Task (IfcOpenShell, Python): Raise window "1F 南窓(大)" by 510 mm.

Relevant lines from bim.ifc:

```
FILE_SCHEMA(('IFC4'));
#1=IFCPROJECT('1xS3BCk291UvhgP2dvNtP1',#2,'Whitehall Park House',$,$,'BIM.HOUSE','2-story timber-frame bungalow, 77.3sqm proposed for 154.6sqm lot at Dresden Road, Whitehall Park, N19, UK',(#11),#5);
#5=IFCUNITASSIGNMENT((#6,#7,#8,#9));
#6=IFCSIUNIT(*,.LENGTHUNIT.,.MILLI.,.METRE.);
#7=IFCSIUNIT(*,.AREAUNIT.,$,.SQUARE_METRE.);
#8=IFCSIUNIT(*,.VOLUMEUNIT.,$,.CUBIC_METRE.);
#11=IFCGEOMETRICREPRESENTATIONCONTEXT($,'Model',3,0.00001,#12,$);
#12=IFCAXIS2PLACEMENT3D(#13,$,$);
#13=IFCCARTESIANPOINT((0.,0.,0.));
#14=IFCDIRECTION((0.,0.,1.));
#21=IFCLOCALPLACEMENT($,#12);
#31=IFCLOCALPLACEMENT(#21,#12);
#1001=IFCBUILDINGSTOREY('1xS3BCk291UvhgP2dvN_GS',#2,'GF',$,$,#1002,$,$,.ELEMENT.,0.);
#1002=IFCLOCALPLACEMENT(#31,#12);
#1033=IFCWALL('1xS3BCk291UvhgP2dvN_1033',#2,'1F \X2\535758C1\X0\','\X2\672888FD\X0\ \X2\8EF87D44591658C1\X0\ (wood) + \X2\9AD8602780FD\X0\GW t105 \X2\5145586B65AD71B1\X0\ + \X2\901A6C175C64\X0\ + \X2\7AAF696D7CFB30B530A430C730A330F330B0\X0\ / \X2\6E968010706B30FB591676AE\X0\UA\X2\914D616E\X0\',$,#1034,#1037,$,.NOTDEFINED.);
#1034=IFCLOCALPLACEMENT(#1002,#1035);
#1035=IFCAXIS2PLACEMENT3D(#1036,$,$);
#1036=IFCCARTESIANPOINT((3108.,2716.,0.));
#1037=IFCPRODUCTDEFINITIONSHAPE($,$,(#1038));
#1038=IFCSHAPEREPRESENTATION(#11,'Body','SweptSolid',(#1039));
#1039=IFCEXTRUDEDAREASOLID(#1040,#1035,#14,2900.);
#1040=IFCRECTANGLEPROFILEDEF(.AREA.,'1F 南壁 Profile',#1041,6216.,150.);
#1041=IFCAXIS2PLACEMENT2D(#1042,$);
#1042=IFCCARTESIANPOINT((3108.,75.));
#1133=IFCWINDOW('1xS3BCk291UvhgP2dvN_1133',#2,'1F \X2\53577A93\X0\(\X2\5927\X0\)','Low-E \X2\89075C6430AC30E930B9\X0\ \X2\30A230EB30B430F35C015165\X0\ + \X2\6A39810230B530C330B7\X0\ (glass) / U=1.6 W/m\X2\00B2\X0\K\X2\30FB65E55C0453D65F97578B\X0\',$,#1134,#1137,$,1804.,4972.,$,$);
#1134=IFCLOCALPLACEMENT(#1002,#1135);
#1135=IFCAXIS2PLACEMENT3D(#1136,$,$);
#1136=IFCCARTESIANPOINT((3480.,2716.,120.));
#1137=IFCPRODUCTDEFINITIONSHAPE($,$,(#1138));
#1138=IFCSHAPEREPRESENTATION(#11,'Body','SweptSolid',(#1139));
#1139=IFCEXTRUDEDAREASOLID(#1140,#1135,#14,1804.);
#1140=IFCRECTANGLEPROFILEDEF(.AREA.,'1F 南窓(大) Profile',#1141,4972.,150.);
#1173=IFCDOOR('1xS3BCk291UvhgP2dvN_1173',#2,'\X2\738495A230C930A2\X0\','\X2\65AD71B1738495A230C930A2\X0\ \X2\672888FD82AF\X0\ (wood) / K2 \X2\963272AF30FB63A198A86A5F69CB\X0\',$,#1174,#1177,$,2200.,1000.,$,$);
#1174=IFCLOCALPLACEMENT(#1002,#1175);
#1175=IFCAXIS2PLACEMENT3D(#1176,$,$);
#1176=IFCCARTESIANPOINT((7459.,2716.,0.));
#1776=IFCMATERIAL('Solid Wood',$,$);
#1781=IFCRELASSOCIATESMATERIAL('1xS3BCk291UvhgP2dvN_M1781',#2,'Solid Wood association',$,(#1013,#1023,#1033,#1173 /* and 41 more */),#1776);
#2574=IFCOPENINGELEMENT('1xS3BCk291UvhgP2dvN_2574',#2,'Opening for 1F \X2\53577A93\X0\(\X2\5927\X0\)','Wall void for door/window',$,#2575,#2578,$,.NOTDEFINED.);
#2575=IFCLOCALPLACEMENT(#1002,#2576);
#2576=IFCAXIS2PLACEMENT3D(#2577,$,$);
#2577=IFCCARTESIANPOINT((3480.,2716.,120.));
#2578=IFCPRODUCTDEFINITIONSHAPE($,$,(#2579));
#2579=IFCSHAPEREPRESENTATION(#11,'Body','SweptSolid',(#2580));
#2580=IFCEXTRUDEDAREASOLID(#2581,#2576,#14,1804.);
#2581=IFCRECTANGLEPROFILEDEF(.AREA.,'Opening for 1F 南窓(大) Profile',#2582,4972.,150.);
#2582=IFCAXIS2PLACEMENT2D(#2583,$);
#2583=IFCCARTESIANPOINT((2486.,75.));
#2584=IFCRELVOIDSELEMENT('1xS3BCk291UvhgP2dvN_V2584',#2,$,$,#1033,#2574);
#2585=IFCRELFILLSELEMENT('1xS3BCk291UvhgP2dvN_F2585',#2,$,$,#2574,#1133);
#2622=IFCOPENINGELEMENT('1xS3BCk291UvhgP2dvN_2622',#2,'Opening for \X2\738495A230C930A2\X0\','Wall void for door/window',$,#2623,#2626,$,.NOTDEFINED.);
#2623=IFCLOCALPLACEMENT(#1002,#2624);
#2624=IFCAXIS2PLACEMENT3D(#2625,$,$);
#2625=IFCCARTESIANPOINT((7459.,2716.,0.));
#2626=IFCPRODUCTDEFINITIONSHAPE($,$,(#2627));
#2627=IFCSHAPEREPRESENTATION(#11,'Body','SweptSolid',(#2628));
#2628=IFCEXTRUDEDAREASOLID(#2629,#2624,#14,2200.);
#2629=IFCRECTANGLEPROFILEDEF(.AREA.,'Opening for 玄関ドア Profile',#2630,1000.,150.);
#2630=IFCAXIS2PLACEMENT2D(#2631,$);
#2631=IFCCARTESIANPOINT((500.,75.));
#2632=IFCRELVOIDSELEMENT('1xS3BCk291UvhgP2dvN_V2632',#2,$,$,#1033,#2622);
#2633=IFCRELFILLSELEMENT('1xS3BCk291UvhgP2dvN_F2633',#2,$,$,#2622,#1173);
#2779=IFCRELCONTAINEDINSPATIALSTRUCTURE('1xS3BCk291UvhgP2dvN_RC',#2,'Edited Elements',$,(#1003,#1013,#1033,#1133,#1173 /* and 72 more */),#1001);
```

```python
import numpy as np
import ifcopenshell
import ifcopenshell.api.geometry
import ifcopenshell.util.placement
import ifcopenshell.util.unit

model = ifcopenshell.open("bim.ifc")
unit_scale = ifcopenshell.util.unit.calculate_unit_scale(model)

window = model.by_guid("1xS3BCk291UvhgP2dvN_1133")
opening = window.FillsVoids[0].RelatingOpeningElement
dz = 0.51 / unit_scale

shift = np.array([0.0, 0.0, dz])
# The window is not placed relative to its opening, so move both.
for product in (opening, window):
    matrix = ifcopenshell.util.placement.get_local_placement(product.ObjectPlacement)
    matrix[:3, 3] += shift
    ifcopenshell.api.geometry.edit_object_placement(model, product=product, matrix=matrix, is_si=False)

print(f"moved by {dz * unit_scale:+.3f} m")

model.write("bim_v2.ifc")
```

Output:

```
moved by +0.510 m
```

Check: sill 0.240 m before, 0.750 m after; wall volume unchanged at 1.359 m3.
